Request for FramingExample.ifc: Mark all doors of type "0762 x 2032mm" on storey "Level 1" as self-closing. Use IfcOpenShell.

First a look at what the model holds.

```python
import ifcopenshell
import ifcopenshell.util.element

model = ifcopenshell.open("FramingExample.ifc")
print(model.schema)
storey = next(s for s in model.by_type("IfcBuildingStorey") if s.Name == "Level 1")
doors = [e for e in ifcopenshell.util.element.get_decomposition(storey) if e.is_a("IfcDoor")]
seen = {}
for e in doors:
    element_type = ifcopenshell.util.element.get_type(e)
    key = (element_type.Name if element_type != e and element_type else None, ifcopenshell.util.element.get_pset(e, "Pset_DoorCommon", "SelfClosing"))
    seen[key] = seen.get(key, 0) + 1
for (name, value), count in sorted(seen.items(), key=str):
    print(count, "x", name, "|", value)
```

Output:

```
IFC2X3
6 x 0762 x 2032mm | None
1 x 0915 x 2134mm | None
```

```python
import ifcopenshell
import ifcopenshell.api.pset
import ifcopenshell.util.element

model = ifcopenshell.open("FramingExample.ifc")

storey = next(s for s in model.by_type("IfcBuildingStorey") if s.Name == "Level 1")
doors = [e for e in ifcopenshell.util.element.get_decomposition(storey) if e.is_a("IfcDoor")]

count = 0
for e in doors:
    element_type = ifcopenshell.util.element.get_type(e)
    if element_type in (None, e) or element_type.Name != "0762 x 2032mm":
        continue
    # add_pset returns the element's existing set when there is one.
    pset = ifcopenshell.api.pset.add_pset(model, product=e, name="Pset_DoorCommon")
    ifcopenshell.api.pset.edit_pset(model, pset=pset, properties={"SelfClosing": True})
    count += 1

print(count, "doors updated")

model.write("FramingExample_updated.ifc")
```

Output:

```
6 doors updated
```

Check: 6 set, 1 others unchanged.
